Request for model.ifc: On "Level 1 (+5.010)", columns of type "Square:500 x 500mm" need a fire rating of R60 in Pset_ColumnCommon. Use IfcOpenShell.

First a look at what the model holds.

```python
import ifcopenshell
import ifcopenshell.util.element

model = ifcopenshell.open("model.ifc")
print(model.schema)
storey = next(s for s in model.by_type("IfcBuildingStorey") if s.Name == "Level 1 (+5.010)")
columns = [e for e in ifcopenshell.util.element.get_decomposition(storey) if e.is_a("IfcColumn")]
seen = {}
for e in columns:
    element_type = ifcopenshell.util.element.get_type(e)
    key = (element_type.Name if element_type != e and element_type else None, ifcopenshell.util.element.get_pset(e, "Pset_ColumnCommon", "FireRating"))
    seen[key] = seen.get(key, 0) + 1
for (name, value), count in sorted(seen.items(), key=str):
    print(count, "x", name, "|", value)
```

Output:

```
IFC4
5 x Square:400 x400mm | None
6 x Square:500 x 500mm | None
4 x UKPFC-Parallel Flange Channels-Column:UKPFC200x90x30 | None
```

```python
import ifcopenshell
import ifcopenshell.api.pset
import ifcopenshell.util.element

model = ifcopenshell.open("model.ifc")

storey = next(s for s in model.by_type("IfcBuildingStorey") if s.Name == "Level 1 (+5.010)")
columns = [e for e in ifcopenshell.util.element.get_decomposition(storey) if e.is_a("IfcColumn")]

count = 0
for e in columns:
    element_type = ifcopenshell.util.element.get_type(e)
    if element_type in (None, e) or element_type.Name != "Square:500 x 500mm":
        continue
    # add_pset returns the element's existing set when there is one.
    pset = ifcopenshell.api.pset.add_pset(model, product=e, name="Pset_ColumnCommon")
    ifcopenshell.api.pset.edit_pset(model, pset=pset, properties={"FireRating": "R60"})
    count += 1

print(count, "columns updated")

model.write("model_edited.ifc")
```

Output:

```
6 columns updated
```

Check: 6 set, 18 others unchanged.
